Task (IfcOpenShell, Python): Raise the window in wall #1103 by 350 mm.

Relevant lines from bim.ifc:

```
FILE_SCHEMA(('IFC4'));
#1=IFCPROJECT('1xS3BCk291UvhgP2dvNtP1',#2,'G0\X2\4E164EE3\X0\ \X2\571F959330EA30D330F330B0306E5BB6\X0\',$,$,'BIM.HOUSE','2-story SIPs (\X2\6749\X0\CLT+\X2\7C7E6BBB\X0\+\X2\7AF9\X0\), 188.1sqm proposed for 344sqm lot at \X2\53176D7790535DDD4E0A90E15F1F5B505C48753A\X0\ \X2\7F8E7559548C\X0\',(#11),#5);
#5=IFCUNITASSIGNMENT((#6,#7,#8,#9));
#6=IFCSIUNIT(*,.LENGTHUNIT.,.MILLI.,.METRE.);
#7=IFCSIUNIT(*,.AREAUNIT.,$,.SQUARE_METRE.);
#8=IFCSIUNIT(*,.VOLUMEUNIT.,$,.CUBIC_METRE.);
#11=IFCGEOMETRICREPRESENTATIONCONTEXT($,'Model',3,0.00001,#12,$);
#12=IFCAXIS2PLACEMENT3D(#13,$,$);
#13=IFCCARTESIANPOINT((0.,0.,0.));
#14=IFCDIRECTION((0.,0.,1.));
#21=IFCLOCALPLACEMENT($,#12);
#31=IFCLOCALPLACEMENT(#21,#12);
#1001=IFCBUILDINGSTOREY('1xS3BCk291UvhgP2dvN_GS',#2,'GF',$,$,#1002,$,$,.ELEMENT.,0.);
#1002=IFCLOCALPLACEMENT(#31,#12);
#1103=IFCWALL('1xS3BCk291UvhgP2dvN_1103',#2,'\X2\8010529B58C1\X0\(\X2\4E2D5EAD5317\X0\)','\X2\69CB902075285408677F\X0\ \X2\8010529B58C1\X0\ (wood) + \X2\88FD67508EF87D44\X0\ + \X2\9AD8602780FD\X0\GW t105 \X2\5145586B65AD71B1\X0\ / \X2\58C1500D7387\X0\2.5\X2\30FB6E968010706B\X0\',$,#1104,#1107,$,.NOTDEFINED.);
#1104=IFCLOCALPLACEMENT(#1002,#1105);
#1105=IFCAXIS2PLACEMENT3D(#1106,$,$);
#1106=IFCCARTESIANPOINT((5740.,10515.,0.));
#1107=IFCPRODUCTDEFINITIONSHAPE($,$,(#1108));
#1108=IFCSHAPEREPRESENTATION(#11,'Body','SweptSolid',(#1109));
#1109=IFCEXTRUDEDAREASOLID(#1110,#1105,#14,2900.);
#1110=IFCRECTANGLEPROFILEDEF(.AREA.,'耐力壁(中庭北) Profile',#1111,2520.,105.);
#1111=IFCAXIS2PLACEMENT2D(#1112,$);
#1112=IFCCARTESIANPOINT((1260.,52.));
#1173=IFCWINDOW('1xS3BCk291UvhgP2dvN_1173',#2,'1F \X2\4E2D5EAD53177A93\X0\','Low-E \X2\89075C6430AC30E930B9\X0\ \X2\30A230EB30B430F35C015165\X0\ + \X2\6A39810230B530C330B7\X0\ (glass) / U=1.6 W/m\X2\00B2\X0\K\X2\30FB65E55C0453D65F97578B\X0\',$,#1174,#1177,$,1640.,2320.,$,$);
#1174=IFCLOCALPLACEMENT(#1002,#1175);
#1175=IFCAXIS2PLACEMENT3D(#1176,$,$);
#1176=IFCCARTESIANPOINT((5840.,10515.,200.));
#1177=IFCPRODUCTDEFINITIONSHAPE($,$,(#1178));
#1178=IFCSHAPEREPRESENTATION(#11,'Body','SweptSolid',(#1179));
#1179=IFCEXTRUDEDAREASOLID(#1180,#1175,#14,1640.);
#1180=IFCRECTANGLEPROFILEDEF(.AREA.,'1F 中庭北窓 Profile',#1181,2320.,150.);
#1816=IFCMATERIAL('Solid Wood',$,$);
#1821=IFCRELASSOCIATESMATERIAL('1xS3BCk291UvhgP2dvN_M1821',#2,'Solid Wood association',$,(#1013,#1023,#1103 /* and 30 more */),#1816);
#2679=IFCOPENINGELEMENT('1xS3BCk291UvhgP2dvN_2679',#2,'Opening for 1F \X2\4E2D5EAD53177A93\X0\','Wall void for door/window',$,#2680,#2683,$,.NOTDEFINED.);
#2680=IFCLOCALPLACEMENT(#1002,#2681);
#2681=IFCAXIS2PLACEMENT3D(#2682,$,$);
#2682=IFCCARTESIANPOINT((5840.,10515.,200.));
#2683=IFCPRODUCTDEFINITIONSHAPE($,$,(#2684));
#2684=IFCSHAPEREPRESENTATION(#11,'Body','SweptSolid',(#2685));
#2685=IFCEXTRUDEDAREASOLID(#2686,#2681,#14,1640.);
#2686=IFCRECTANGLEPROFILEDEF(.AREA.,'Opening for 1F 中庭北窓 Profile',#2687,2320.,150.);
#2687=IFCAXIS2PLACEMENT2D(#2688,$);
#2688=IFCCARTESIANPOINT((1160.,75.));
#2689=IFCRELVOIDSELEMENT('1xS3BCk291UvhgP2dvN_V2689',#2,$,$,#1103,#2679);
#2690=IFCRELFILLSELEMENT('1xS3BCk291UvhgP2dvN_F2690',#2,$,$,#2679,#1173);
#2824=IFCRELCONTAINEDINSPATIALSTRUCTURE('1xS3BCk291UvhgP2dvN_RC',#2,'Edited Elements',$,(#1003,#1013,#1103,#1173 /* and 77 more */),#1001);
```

```python
import numpy as np
import ifcopenshell
import ifcopenshell.api.geometry
import ifcopenshell.util.placement
import ifcopenshell.util.unit

model = ifcopenshell.open("bim.ifc")
unit_scale = ifcopenshell.util.unit.calculate_unit_scale(model)

window = model.by_guid("1xS3BCk291UvhgP2dvN_1173")
opening = window.FillsVoids[0].RelatingOpeningElement
dz = 0.35 / unit_scale

shift = np.array([0.0, 0.0, dz])
# The window is not placed relative to its opening, so move both.
for product in (opening, window):
    matrix = ifcopenshell.util.placement.get_local_placement(product.ObjectPlacement)
    matrix[:3, 3] += shift
    ifcopenshell.api.geometry.edit_object_placement(model, product=product, matrix=matrix, is_si=False)

print(f"moved by {dz * unit_scale:+.3f} m")

model.write("bim_rev.ifc")
```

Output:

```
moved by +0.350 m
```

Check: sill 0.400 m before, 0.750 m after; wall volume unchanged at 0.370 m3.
